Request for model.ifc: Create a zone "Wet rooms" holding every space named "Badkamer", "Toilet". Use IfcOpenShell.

First a look at what the model holds.

```python
import ifcopenshell

model = ifcopenshell.open("model.ifc")
print(model.schema)
seen = {}
for space in model.by_type("IfcSpace"):
    seen[space.LongName] = seen.get(space.LongName, 0) + 1
for name, count in sorted(seen.items(), key=str):
    print(count, "x", name)
print("zones:", [z.Name for z in model.by_type("IfcZone")][:20])
```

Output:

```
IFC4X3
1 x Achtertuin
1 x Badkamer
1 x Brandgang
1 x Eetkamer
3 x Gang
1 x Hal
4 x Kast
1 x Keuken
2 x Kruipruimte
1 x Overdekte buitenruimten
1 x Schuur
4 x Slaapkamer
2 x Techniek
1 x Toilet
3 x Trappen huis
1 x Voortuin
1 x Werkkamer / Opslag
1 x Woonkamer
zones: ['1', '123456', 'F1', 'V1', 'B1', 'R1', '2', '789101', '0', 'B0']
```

```python
import ifcopenshell
import ifcopenshell.api.group
import ifcopenshell.api.root

model = ifcopenshell.open("model.ifc")

names = {"Badkamer", "Toilet"}
spaces = [s for s in model.by_type("IfcSpace") if s.LongName in names]

zone = ifcopenshell.api.root.create_entity(model, ifc_class="IfcZone", name="Wet rooms")
ifcopenshell.api.group.assign_group(model, products=spaces, group=zone)
print(len(spaces), "spaces in", zone.Name)

model.write("model-out.ifc")
```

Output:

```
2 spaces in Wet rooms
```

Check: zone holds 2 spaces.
